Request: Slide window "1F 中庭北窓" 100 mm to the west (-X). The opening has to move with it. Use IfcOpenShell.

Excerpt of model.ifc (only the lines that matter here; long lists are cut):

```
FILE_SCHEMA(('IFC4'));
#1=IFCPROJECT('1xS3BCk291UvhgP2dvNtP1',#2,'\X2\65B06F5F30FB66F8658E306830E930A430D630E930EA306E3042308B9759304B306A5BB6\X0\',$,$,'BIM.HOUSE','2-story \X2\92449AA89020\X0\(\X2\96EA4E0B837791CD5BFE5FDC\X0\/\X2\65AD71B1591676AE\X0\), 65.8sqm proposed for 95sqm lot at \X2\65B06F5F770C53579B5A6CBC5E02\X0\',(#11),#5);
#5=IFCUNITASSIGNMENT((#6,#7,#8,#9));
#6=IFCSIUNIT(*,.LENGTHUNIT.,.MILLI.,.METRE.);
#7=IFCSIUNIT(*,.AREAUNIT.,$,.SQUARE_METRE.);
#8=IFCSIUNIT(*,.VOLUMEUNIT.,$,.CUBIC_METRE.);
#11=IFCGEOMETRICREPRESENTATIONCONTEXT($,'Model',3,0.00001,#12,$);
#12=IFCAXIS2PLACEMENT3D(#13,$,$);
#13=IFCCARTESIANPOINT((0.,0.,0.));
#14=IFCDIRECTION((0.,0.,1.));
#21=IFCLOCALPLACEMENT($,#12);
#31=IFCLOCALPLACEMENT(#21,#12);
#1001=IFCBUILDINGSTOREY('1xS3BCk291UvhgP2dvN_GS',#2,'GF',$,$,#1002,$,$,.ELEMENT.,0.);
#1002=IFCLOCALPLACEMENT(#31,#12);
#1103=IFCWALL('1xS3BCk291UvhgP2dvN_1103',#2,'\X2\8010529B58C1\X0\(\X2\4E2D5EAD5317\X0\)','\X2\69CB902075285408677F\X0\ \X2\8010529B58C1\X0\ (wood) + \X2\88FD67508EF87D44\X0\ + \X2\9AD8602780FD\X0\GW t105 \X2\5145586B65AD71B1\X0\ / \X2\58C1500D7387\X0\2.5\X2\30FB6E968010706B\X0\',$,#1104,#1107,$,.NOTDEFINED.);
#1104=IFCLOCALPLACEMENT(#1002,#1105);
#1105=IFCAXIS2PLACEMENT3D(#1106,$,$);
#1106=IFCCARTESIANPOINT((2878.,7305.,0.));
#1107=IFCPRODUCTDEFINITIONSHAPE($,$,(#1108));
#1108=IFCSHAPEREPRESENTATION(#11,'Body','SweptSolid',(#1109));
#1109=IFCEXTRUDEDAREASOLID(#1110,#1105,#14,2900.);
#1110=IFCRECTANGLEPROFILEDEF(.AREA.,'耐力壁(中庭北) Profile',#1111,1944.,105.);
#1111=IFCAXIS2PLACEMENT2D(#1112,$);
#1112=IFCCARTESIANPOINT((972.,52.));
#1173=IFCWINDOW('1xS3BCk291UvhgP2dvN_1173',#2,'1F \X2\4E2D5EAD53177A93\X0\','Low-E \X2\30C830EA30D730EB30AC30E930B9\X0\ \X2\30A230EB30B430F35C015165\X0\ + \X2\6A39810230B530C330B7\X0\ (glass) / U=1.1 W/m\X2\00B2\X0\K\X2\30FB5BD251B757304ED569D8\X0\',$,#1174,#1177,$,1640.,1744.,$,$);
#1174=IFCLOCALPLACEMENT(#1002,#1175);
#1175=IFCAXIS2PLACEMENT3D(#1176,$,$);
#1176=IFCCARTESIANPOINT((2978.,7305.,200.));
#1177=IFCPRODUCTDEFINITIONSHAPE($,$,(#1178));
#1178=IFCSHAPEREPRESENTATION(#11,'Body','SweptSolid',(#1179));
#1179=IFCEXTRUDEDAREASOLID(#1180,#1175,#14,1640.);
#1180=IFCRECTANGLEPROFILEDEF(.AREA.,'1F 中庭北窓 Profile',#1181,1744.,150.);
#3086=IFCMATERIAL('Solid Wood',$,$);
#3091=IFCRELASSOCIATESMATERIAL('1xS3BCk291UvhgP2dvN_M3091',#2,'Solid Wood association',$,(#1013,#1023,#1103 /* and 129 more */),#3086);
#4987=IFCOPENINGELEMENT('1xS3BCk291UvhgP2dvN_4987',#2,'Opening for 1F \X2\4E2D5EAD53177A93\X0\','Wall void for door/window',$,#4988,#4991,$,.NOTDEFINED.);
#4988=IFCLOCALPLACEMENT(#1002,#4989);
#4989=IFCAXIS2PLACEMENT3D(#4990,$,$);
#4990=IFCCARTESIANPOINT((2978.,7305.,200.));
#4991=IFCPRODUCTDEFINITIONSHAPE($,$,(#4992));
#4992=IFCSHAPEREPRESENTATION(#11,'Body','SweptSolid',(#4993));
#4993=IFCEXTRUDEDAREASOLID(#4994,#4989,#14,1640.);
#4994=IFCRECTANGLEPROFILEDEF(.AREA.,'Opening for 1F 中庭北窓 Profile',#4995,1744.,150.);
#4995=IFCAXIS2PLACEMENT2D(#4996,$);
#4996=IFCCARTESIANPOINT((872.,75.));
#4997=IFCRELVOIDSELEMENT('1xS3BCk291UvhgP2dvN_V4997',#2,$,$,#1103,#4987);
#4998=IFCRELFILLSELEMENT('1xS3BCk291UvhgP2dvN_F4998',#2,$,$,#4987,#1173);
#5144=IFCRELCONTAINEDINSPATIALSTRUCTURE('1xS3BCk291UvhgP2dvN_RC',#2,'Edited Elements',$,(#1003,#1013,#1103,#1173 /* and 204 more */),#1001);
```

```python
import ifcopenshell
import ifcopenshell.api.geometry
import ifcopenshell.util.placement
import ifcopenshell.util.unit

model = ifcopenshell.open("model.ifc")
unit_scale = ifcopenshell.util.unit.calculate_unit_scale(model)

window = model.by_guid("1xS3BCk291UvhgP2dvN_1173")
opening = window.FillsVoids[0].RelatingOpeningElement
wall = opening.VoidsElements[0].RelatingBuildingElement

wall_matrix = ifcopenshell.util.placement.get_local_placement(wall.ObjectPlacement)
shift = wall_matrix[:3, 0] * -0.1 / unit_scale
before = ifcopenshell.util.placement.get_local_placement(window.ObjectPlacement)[:3, 3].copy()

# The window is not placed relative to its opening, so move both.
for product in (opening, window):
    matrix = ifcopenshell.util.placement.get_local_placement(product.ObjectPlacement)
    matrix[:3, 3] += shift
    ifcopenshell.api.geometry.edit_object_placement(model, product=product, matrix=matrix, is_si=False)

after = ifcopenshell.util.placement.get_local_placement(window.ObjectPlacement)[:3, 3]
print("window moved by", (after - before).round(3) + 0.0)

model.write("model_rev.ifc")
```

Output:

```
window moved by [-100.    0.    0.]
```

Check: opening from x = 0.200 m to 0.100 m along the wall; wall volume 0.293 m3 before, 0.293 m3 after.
